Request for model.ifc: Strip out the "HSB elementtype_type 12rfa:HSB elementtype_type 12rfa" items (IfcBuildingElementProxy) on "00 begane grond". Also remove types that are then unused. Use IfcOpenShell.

First a look at what the model holds.

```python
import ifcopenshell
import ifcopenshell.util.element

model = ifcopenshell.open("model.ifc")
print(model.schema)
storey = next(s for s in model.by_type("IfcBuildingStorey") if s.Name == "00 begane grond")
proxies = [e for e in ifcopenshell.util.element.get_decomposition(storey) if e.is_a("IfcBuildingElementProxy")]
seen = {}
for e in proxies:
    element_type = ifcopenshell.util.element.get_type(e)
    name = element_type.Name if element_type not in (None, e) else None
    seen[name] = seen.get(name, 0) + 1
for name, count in sorted(seen.items(), key=str):
    print(count, "x", name)
```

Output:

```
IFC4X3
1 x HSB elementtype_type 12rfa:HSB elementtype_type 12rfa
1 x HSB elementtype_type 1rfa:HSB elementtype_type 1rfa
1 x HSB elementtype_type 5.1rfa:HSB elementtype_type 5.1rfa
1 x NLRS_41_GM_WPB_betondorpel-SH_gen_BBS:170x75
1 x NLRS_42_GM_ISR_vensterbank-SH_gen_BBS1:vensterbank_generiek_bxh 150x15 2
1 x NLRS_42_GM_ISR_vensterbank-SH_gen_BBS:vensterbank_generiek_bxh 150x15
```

```python
import ifcopenshell
import ifcopenshell.api.root
import ifcopenshell.util.element

model = ifcopenshell.open("model.ifc")

storey = next(s for s in model.by_type("IfcBuildingStorey") if s.Name == "00 begane grond")
proxies = [e for e in ifcopenshell.util.element.get_decomposition(storey) if e.is_a("IfcBuildingElementProxy")]
targets = [e for e in proxies if (t := ifcopenshell.util.element.get_type(e)) not in (None, e) and t.Name == "HSB elementtype_type 12rfa:HSB elementtype_type 12rfa"]
types = {ifcopenshell.util.element.get_type(e) for e in targets} - {None, *targets}

for e in targets:
    ifcopenshell.api.root.remove_product(model, product=e)
print(len(targets), "removed")

unused = [t for t in types if not ifcopenshell.util.element.get_types(t)]
for t in unused:
    ifcopenshell.api.root.remove_product(model, product=t)
print(len(unused), "unused types removed")

model.write("model_rev.ifc")
```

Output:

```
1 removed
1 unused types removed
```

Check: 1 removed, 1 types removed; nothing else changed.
